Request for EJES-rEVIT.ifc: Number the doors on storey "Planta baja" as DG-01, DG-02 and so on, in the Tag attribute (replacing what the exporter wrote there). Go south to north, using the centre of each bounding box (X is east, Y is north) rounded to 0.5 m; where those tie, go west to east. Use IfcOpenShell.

First a look at what the model holds.

```python
import ifcopenshell
import ifcopenshell.util.element
import ifcopenshell.util.placement

model = ifcopenshell.open("EJES-rEVIT.ifc")
print(model.schema)
storey = next(s for s in model.by_type("IfcBuildingStorey") if s.Name == "Planta baja")
doors = [e for e in ifcopenshell.util.element.get_decomposition(storey) if e.is_a("IfcDoor")]
for e in sorted(doors, key=lambda e: e.id()):
    origin = ifcopenshell.util.placement.get_local_placement(e.ObjectPlacement)[:3, 3]
    print(e.id(), e.Tag, e.Name, origin.round(2) + 0.0, sep=" | ")
```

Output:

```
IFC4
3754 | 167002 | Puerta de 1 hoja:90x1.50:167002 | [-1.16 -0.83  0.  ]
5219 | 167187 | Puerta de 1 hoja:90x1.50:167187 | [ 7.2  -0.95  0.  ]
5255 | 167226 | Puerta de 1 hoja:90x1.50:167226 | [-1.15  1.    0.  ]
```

```python
import ifcopenshell
import ifcopenshell.geom
import ifcopenshell.util.element
import ifcopenshell.util.shape

model = ifcopenshell.open("EJES-rEVIT.ifc")
settings = ifcopenshell.geom.settings()
settings.set("use-world-coords", True)


def centre(element):
    shape = ifcopenshell.geom.create_shape(settings, element)
    return ifcopenshell.util.shape.get_bbox_centroid(shape.geometry)


storey = next(s for s in model.by_type("IfcBuildingStorey") if s.Name == "Planta baja")
doors = [e for e in ifcopenshell.util.element.get_decomposition(storey) if e.is_a("IfcDoor")]

# Insertion points can sit at a corner or the storey origin, so sort by the geometry (in metres).
centres = {e: centre(e) for e in doors}
doors.sort(key=lambda e: (round(centres[e][1] / 0.5), centres[e][0]))

for i, e in enumerate(doors, start=1):
    number = f"DG-{i:02d}"
    e.Tag = number
    print(e.id(), number)

model.write("EJES-rEVIT_edited.ifc")
```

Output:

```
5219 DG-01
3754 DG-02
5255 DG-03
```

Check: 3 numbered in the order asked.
